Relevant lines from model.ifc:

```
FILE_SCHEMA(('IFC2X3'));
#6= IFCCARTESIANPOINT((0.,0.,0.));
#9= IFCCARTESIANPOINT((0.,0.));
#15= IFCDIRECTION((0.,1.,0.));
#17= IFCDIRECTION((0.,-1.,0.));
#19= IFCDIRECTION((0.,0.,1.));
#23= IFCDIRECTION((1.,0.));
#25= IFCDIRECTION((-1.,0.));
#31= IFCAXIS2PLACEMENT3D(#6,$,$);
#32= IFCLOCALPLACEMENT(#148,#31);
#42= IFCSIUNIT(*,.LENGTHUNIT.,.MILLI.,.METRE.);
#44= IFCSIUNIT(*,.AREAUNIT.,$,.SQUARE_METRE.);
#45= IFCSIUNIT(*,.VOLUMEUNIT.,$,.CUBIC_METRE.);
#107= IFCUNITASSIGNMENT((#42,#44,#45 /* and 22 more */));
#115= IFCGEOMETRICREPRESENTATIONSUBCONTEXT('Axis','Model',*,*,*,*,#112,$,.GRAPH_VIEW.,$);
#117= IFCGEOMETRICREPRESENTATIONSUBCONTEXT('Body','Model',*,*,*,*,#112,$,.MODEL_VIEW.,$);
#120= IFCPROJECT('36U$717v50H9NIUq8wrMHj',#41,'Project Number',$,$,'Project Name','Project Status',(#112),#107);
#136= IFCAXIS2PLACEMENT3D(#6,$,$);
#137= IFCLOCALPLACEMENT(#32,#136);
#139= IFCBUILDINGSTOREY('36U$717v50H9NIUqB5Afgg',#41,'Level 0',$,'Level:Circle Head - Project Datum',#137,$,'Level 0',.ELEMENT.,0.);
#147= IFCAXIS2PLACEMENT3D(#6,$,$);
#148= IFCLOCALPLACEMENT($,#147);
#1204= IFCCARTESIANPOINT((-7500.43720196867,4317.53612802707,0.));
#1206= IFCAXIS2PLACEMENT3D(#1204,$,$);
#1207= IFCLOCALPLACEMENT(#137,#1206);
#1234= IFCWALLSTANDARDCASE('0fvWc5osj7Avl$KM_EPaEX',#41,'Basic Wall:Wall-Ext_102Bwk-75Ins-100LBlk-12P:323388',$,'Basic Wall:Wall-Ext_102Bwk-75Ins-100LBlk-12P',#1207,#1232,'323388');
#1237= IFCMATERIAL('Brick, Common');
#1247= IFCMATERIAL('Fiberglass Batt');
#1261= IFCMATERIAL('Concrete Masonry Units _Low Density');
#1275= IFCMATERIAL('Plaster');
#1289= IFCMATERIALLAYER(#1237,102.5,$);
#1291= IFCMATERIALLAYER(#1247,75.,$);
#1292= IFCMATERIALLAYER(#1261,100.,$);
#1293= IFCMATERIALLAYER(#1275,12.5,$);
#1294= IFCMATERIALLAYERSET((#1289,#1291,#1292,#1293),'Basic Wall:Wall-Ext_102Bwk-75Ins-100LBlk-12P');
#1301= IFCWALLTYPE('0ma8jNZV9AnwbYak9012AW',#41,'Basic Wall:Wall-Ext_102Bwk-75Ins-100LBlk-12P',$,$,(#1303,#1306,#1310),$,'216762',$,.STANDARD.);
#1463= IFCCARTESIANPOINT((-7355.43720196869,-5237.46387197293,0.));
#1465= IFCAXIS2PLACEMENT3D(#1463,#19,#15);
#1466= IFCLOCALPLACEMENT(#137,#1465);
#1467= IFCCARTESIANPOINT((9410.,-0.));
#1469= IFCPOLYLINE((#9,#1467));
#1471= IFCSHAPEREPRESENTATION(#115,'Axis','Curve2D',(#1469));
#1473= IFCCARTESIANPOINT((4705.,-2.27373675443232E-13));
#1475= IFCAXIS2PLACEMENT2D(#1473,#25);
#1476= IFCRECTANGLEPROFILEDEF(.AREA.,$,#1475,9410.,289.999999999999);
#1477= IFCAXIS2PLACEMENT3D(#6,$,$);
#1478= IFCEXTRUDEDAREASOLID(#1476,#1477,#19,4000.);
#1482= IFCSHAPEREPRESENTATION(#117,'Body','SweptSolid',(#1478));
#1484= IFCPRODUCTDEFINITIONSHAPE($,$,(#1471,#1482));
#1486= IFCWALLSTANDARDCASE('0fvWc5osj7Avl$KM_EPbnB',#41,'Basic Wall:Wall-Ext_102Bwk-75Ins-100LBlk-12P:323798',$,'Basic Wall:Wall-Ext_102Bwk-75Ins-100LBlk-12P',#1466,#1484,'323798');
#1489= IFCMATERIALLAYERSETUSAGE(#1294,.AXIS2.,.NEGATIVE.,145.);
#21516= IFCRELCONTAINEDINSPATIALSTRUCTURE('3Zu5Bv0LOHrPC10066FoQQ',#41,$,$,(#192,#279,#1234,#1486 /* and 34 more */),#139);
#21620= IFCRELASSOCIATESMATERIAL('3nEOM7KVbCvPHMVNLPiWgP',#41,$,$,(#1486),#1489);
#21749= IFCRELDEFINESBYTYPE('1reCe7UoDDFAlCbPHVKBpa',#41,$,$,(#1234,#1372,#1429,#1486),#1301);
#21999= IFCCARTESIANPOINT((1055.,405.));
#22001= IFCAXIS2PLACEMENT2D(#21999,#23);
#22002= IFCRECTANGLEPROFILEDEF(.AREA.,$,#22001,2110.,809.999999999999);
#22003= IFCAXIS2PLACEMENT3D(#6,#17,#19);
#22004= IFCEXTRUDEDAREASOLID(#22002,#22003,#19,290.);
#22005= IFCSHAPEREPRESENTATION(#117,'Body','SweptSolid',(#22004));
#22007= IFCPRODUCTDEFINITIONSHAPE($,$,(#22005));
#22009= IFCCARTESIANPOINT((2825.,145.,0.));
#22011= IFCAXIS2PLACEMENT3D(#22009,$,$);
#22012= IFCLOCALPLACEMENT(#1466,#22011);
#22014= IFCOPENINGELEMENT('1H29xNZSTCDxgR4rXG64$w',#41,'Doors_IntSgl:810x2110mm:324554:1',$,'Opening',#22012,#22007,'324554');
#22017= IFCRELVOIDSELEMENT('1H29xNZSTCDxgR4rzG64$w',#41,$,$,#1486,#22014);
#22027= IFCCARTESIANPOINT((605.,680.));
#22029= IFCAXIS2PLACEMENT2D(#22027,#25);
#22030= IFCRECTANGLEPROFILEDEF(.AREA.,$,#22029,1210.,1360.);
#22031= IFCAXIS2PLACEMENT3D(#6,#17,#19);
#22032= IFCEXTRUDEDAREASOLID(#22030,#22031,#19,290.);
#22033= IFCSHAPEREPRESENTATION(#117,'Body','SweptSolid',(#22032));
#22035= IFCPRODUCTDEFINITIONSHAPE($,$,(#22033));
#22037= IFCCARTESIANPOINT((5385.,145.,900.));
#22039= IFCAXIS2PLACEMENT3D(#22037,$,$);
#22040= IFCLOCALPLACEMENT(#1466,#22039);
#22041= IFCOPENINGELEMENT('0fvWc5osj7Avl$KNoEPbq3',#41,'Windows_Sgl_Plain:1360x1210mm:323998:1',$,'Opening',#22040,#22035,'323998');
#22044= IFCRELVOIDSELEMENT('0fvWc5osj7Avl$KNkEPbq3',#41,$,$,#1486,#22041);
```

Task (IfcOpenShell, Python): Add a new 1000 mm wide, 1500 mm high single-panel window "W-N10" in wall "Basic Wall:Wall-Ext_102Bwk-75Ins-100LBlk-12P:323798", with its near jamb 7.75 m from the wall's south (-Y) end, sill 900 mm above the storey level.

```python
import numpy as np
import ifcopenshell
import ifcopenshell.api.feature
import ifcopenshell.api.geometry
import ifcopenshell.api.root
import ifcopenshell.api.spatial
import ifcopenshell.api.type
import ifcopenshell.geom
import ifcopenshell.util.element
import ifcopenshell.util.placement
import ifcopenshell.util.representation
import ifcopenshell.util.shape
import ifcopenshell.util.unit

model = ifcopenshell.open("model.ifc")
unit_scale = ifcopenshell.util.unit.calculate_unit_scale(model)
settings = ifcopenshell.geom.settings()


def volume(element):
    """Net volume in cubic metres, openings subtracted."""
    shape = ifcopenshell.geom.create_shape(settings, element)
    return ifcopenshell.util.shape.get_volume(shape.geometry)


wall = model.by_guid("0fvWc5osj7Avl$KM_EPbnB")
storey = ifcopenshell.util.element.get_container(wall, ifc_class="IfcBuildingStorey")
context = ifcopenshell.util.representation.get_context(model, "Model", "Body", "MODEL_VIEW")
before = volume(wall)

width, height, from_end, sill = 1, 1.5, 7.75, 0.9  # metres

# The wall runs along its own X axis, and the end named is its -X end.
wall_shape = ifcopenshell.geom.create_shape(settings, wall)
x, y, z = ifcopenshell.util.shape.get_vertices(wall_shape.geometry).T
start = x.min() + from_end
face, thickness = float(y.min()), float(y.max() - y.min())
wall_matrix = ifcopenshell.util.placement.get_local_placement(wall.ObjectPlacement)
level = ifcopenshell.util.placement.get_local_placement(storey.ObjectPlacement)[2, 3]


def in_wall(x, y):
    """Placement at x, y metres in the wall's axes, at sill height."""
    matrix = wall_matrix.copy()
    matrix[:, 3] = wall_matrix @ np.array([x / unit_scale, y / unit_scale, 0.0, 1.0])
    matrix[2, 3] = level + sill / unit_scale
    return matrix


# Opening: a box that overshoots both wall faces by 50 mm.
opening = ifcopenshell.api.root.create_entity(model, ifc_class="IfcOpeningElement")
box = ifcopenshell.api.geometry.add_wall_representation(
    model, context=context, length=width, height=height, thickness=thickness + 0.1
)
ifcopenshell.api.geometry.assign_representation(model, product=opening, representation=box)
ifcopenshell.api.geometry.edit_object_placement(model, product=opening, matrix=in_wall(start, face - 0.05), is_si=False)
ifcopenshell.api.feature.add_feature(model, feature=opening, element=wall)

window = ifcopenshell.api.root.create_entity(model, ifc_class="IfcWindow", name="W-N10")
window.OverallWidth, window.OverallHeight = width / unit_scale, height / unit_scale
body = ifcopenshell.api.geometry.add_window_representation(
    model,
    context=context,
    overall_width=window.OverallWidth,
    overall_height=window.OverallHeight,
    partition_type="SINGLE_PANEL",
)
ifcopenshell.api.geometry.assign_representation(model, product=window, representation=body)
ifcopenshell.api.spatial.assign_container(model, products=[window], relating_structure=storey)
fills = ifcopenshell.api.feature.add_filling(model, opening=opening, element=window)
fills.OwnerHistory = window.OwnerHistory  # required in IFC2X3

# IFC2X3 keeps the operation on the window style.
style = ifcopenshell.api.root.create_entity(model, ifc_class="IfcWindowStyle", name="W-N10")
style.OperationType, style.ConstructionType = "SINGLE_PANEL", "NOTDEFINED"
style.ParameterTakesPrecedence = style.Sizeable = False
ifcopenshell.api.type.assign_type(model, related_objects=[window], relating_type=style)

# Centre the window in the wall's thickness.
ifcopenshell.api.geometry.edit_object_placement(model, product=window, matrix=in_wall(start, face), is_si=False)
window_shape = ifcopenshell.geom.create_shape(settings, window)
depth = ifcopenshell.util.shape.get_vertices(window_shape.geometry)[:, 1]
offset = face + thickness / 2 - (depth.min() + depth.max()) / 2
ifcopenshell.api.geometry.edit_object_placement(model, product=window, matrix=in_wall(start, offset), is_si=False)

after = volume(wall)

print(f"wall volume {before:.3f} -> {after:.3f} m3")

model.write("model_v2.ifc")
```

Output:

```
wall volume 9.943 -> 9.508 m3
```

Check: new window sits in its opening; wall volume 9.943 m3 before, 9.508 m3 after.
